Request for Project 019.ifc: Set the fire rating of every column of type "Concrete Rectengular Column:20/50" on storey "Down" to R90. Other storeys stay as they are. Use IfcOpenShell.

First a look at what the model holds.

```python
import ifcopenshell
import ifcopenshell.util.element

model = ifcopenshell.open("Project 019.ifc")
print(model.schema)
storey = next(s for s in model.by_type("IfcBuildingStorey") if s.Name == "Down")
columns = [e for e in ifcopenshell.util.element.get_decomposition(storey) if e.is_a("IfcColumn")]
seen = {}
for e in columns:
    element_type = ifcopenshell.util.element.get_type(e)
    key = (element_type.Name if element_type != e and element_type else None, ifcopenshell.util.element.get_pset(e, "Pset_ColumnCommon", "FireRating"))
    seen[key] = seen.get(key, 0) + 1
for (name, value), count in sorted(seen.items(), key=str):
    print(count, "x", name, "|", value)
```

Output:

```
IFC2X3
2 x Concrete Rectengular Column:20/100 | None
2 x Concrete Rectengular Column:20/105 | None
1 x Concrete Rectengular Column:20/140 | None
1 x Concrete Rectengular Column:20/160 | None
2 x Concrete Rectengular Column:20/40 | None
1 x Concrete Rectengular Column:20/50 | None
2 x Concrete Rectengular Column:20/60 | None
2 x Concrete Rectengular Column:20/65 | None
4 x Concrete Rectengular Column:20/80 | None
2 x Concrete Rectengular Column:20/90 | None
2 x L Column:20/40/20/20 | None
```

```python
import ifcopenshell
import ifcopenshell.api.pset
import ifcopenshell.util.element

model = ifcopenshell.open("Project 019.ifc")

storey = next(s for s in model.by_type("IfcBuildingStorey") if s.Name == "Down")
columns = [e for e in ifcopenshell.util.element.get_decomposition(storey) if e.is_a("IfcColumn")]

count = 0
for e in columns:
    element_type = ifcopenshell.util.element.get_type(e)
    if element_type in (None, e) or element_type.Name != "Concrete Rectengular Column:20/50":
        continue
    # add_pset returns the element's existing set when there is one.
    pset = ifcopenshell.api.pset.add_pset(model, product=e, name="Pset_ColumnCommon")
    ifcopenshell.api.pset.edit_pset(model, pset=pset, properties={"FireRating": "R90"})
    count += 1

print(count, "columns updated")

model.write("Project 019_edited.ifc")
```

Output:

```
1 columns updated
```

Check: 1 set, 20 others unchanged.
